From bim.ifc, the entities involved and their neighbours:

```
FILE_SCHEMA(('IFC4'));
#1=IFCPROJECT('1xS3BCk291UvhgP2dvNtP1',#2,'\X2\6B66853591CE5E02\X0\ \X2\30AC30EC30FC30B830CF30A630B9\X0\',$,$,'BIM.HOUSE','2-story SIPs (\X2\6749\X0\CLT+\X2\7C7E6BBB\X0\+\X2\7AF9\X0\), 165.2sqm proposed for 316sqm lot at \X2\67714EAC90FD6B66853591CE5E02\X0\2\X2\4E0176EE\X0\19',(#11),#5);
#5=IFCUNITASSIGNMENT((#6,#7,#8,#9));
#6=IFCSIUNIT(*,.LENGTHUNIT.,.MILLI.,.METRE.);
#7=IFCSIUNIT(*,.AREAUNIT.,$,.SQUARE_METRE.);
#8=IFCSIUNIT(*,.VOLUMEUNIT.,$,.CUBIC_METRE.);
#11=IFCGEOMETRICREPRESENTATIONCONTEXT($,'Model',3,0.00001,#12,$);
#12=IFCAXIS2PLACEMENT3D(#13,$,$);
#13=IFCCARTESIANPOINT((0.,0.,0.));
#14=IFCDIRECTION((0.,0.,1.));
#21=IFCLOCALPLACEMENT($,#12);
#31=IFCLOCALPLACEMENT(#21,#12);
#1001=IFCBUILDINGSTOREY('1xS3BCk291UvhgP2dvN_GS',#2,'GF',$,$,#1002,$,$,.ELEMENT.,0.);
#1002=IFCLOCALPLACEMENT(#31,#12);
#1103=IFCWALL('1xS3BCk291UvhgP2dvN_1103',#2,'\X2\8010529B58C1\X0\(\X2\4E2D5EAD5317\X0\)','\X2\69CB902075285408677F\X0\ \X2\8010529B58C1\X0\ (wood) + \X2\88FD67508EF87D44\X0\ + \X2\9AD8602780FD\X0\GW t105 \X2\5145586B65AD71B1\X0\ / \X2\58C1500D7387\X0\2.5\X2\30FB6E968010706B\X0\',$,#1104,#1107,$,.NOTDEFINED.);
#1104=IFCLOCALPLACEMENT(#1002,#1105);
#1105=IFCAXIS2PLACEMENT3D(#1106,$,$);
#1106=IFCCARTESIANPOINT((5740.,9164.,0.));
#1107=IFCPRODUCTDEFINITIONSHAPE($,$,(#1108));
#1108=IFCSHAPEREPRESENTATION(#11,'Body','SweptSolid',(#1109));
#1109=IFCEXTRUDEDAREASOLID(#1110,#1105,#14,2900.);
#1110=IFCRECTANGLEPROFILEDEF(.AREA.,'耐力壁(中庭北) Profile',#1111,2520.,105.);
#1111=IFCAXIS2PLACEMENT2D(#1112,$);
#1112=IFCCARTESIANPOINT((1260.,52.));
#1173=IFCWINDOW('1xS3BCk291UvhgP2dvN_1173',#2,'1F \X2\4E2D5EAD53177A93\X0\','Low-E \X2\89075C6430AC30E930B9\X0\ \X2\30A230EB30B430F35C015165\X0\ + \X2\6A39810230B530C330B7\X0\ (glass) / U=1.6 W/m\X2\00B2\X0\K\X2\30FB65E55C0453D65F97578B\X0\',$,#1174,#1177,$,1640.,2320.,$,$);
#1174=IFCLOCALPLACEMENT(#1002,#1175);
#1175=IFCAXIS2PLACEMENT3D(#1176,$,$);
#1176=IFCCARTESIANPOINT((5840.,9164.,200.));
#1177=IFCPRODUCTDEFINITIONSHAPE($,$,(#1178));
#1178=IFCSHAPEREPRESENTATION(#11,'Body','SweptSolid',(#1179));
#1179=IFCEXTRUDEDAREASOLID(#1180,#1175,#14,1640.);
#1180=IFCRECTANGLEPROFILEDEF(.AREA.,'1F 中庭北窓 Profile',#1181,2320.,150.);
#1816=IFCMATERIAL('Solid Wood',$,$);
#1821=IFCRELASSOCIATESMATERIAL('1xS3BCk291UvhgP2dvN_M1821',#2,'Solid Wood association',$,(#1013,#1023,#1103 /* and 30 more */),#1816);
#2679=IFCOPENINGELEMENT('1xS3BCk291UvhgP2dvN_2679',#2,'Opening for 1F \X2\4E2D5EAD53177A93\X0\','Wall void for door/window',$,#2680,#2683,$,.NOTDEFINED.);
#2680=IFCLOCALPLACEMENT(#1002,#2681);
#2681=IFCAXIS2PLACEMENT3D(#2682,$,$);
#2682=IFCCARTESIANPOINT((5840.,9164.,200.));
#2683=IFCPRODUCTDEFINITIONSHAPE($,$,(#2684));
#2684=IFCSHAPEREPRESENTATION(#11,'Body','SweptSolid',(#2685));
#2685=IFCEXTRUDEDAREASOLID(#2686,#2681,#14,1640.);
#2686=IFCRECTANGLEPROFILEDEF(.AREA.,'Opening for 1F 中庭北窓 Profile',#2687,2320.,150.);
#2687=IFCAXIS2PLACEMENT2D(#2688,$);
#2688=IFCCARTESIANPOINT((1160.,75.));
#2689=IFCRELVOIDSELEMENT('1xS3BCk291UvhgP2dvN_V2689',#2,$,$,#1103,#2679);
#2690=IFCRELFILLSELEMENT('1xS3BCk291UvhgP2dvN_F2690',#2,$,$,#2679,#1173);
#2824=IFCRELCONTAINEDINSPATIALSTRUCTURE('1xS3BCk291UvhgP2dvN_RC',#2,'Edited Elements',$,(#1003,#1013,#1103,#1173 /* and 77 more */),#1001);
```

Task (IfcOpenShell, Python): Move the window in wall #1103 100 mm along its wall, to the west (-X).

```python
import ifcopenshell
import ifcopenshell.api.geometry
import ifcopenshell.util.placement
import ifcopenshell.util.unit

model = ifcopenshell.open("bim.ifc")
unit_scale = ifcopenshell.util.unit.calculate_unit_scale(model)

window = model.by_guid("1xS3BCk291UvhgP2dvN_1173")
opening = window.FillsVoids[0].RelatingOpeningElement
wall = opening.VoidsElements[0].RelatingBuildingElement

wall_matrix = ifcopenshell.util.placement.get_local_placement(wall.ObjectPlacement)
shift = wall_matrix[:3, 0] * -0.1 / unit_scale
before = ifcopenshell.util.placement.get_local_placement(window.ObjectPlacement)[:3, 3].copy()

# The window is not placed relative to its opening, so move both.
for product in (opening, window):
    matrix = ifcopenshell.util.placement.get_local_placement(product.ObjectPlacement)
    matrix[:3, 3] += shift
    ifcopenshell.api.geometry.edit_object_placement(model, product=product, matrix=matrix, is_si=False)

after = ifcopenshell.util.placement.get_local_placement(window.ObjectPlacement)[:3, 3]
print("window moved by", (after - before).round(3) + 0.0)

model.write("bim_updated.ifc")
```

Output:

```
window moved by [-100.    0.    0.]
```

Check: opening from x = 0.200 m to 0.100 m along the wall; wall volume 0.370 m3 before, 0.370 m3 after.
